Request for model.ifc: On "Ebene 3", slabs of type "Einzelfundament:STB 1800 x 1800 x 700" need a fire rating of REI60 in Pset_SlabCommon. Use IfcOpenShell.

First a look at what the model holds.

```python
import ifcopenshell
import ifcopenshell.util.element

model = ifcopenshell.open("model.ifc")
print(model.schema)
storey = next(s for s in model.by_type("IfcBuildingStorey") if s.Name == "Ebene 3")
slabs = [e for e in ifcopenshell.util.element.get_decomposition(storey) if e.is_a("IfcSlab")]
seen = {}
for e in slabs:
    element_type = ifcopenshell.util.element.get_type(e)
    key = (element_type.Name if element_type != e and element_type else None, ifcopenshell.util.element.get_pset(e, "Pset_SlabCommon", "FireRating"))
    seen[key] = seen.get(key, 0) + 1
for (name, value), count in sorted(seen.items(), key=str):
    print(count, "x", name, "|", value)
```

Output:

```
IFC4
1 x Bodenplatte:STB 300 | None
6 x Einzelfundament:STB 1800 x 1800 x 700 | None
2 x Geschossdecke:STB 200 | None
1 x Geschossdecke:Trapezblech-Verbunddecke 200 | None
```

```python
import ifcopenshell
import ifcopenshell.api.pset
import ifcopenshell.util.element

model = ifcopenshell.open("model.ifc")

storey = next(s for s in model.by_type("IfcBuildingStorey") if s.Name == "Ebene 3")
slabs = [e for e in ifcopenshell.util.element.get_decomposition(storey) if e.is_a("IfcSlab")]

count = 0
for e in slabs:
    element_type = ifcopenshell.util.element.get_type(e)
    if element_type in (None, e) or element_type.Name != "Einzelfundament:STB 1800 x 1800 x 700":
        continue
    # add_pset returns the element's existing set when there is one.
    pset = ifcopenshell.api.pset.add_pset(model, product=e, name="Pset_SlabCommon")
    ifcopenshell.api.pset.edit_pset(model, pset=pset, properties={"FireRating": "REI60"})
    count += 1

print(count, "slabs updated")

model.write("model-out.ifc")
```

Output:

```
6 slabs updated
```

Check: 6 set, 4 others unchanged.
